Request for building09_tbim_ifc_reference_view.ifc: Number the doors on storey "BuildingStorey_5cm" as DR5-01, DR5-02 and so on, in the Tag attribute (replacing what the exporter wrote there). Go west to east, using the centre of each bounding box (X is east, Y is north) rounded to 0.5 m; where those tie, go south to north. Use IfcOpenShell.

First a look at what the model holds.

```python
import ifcopenshell
import ifcopenshell.util.element
import ifcopenshell.util.placement

model = ifcopenshell.open("building09_tbim_ifc_reference_view.ifc")
print(model.schema)
storey = next(s for s in model.by_type("IfcBuildingStorey") if s.Name == "BuildingStorey_5cm")
doors = [e for e in ifcopenshell.util.element.get_decomposition(storey) if e.is_a("IfcDoor")]
for e in sorted(doors, key=lambda e: e.id()):
    origin = ifcopenshell.util.placement.get_local_placement(e.ObjectPlacement)[:3, 3]
    print(e.id(), e.Tag, e.Name, origin.round(2) + 0.0, sep=" | ")
```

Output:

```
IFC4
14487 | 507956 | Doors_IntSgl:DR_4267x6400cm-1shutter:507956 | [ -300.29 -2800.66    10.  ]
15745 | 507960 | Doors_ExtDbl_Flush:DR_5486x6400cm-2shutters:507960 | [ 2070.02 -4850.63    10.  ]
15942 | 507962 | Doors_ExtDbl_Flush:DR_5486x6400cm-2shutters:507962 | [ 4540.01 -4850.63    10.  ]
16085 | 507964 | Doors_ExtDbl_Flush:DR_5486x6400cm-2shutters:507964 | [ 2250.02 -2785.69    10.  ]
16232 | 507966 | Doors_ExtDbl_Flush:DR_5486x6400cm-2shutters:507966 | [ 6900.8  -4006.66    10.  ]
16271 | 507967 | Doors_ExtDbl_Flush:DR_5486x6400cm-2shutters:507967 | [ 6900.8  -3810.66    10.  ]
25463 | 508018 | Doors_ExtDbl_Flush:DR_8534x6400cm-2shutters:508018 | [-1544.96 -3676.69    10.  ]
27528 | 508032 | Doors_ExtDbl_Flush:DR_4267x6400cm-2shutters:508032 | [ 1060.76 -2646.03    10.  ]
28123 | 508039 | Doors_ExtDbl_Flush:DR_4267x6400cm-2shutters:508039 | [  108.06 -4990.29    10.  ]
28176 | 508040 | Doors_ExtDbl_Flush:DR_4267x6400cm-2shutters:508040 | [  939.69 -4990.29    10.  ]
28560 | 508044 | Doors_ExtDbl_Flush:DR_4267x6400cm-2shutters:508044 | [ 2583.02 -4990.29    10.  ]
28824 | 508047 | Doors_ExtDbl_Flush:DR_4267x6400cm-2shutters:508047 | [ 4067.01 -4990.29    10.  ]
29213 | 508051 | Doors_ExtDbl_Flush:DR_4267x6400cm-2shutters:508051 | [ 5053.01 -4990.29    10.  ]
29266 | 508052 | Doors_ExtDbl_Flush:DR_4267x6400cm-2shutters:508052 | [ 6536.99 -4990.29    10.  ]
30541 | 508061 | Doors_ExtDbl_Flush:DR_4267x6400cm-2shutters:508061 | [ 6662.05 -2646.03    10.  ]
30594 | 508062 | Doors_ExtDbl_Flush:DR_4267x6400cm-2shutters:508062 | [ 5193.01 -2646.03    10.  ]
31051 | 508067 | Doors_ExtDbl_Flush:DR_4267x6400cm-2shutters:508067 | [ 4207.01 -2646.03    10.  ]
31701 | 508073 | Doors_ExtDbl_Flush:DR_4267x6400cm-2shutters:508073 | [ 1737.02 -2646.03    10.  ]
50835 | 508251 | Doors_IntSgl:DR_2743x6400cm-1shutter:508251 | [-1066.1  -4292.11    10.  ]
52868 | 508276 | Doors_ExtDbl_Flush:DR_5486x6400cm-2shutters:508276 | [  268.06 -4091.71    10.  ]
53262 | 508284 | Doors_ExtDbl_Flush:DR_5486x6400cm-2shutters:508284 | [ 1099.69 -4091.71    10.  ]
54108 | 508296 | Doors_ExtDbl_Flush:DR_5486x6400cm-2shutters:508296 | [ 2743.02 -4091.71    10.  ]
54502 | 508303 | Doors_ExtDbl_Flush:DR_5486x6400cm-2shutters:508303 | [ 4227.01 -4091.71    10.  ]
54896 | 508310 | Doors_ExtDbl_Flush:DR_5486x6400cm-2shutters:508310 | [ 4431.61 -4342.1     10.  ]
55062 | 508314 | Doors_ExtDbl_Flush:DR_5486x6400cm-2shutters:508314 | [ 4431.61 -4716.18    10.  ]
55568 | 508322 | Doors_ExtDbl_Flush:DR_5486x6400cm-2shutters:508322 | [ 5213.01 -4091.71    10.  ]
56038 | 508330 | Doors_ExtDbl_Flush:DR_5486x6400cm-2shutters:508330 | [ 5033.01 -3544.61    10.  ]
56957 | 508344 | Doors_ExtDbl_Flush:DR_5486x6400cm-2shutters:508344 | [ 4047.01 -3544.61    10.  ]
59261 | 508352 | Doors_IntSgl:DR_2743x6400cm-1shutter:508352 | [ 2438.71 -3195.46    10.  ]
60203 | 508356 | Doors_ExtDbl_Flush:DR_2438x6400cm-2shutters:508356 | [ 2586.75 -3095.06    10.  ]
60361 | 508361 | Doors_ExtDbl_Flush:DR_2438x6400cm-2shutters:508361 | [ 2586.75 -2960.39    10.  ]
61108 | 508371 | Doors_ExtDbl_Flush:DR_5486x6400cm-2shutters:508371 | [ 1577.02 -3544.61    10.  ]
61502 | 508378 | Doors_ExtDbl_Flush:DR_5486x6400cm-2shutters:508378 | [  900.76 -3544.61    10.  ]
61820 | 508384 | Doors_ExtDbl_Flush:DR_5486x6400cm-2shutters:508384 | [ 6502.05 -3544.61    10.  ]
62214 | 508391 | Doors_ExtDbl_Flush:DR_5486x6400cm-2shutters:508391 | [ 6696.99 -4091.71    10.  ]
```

```python
import ifcopenshell
import ifcopenshell.geom
import ifcopenshell.util.element
import ifcopenshell.util.shape

model = ifcopenshell.open("building09_tbim_ifc_reference_view.ifc")
settings = ifcopenshell.geom.settings()
settings.set("use-world-coords", True)


def centre(element):
    shape = ifcopenshell.geom.create_shape(settings, element)
    return ifcopenshell.util.shape.get_bbox_centroid(shape.geometry)


storey = next(s for s in model.by_type("IfcBuildingStorey") if s.Name == "BuildingStorey_5cm")
doors = [e for e in ifcopenshell.util.element.get_decomposition(storey) if e.is_a("IfcDoor")]

# Insertion points can sit at a corner or the storey origin, so sort by the geometry (in metres).
centres = {e: centre(e) for e in doors}
doors.sort(key=lambda e: (round(centres[e][0] / 0.5), centres[e][1]))

for i, e in enumerate(doors, start=1):
    number = f"DR5-{i:02d}"
    e.Tag = number
    print(e.id(), number)

model.write("building09_tbim_ifc_reference_view_updated.ifc")
```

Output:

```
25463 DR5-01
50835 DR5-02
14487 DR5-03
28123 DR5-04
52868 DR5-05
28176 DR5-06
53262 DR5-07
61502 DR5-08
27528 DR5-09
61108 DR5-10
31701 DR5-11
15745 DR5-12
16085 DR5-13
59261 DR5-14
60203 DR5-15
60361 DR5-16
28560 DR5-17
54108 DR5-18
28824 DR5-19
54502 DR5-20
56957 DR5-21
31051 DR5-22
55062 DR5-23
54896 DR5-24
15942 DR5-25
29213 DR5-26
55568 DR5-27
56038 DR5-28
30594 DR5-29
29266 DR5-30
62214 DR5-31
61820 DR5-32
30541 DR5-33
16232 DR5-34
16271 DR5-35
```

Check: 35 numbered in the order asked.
